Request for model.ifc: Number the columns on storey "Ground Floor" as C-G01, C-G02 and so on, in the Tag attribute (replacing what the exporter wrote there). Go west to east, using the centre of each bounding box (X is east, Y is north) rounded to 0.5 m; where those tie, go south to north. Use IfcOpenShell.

First a look at what the model holds.

```python
import ifcopenshell
import ifcopenshell.util.element
import ifcopenshell.util.placement

model = ifcopenshell.open("model.ifc")
print(model.schema)
storey = next(s for s in model.by_type("IfcBuildingStorey") if s.Name == "Ground Floor")
columns = [e for e in ifcopenshell.util.element.get_decomposition(storey) if e.is_a("IfcColumn")]
for e in sorted(columns, key=lambda e: e.id()):
    origin = ifcopenshell.util.placement.get_local_placement(e.ObjectPlacement)[:3, 3]
    print(e.id(), e.Tag, e.Name, origin.round(2) + 0.0, sep=" | ")
```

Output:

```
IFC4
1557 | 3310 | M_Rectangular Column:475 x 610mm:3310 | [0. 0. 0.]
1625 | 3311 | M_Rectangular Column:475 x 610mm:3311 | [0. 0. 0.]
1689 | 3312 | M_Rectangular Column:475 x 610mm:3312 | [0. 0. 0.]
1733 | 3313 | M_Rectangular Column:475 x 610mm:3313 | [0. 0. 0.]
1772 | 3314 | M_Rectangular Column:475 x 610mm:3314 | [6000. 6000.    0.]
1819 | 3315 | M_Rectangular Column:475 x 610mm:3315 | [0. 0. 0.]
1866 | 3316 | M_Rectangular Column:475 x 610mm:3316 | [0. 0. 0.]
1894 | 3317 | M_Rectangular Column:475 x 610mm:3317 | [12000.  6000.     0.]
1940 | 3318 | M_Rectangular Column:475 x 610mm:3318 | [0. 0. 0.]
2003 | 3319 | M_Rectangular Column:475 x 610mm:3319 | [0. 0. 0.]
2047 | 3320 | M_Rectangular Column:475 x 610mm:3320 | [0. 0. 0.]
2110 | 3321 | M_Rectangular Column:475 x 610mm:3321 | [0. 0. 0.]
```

```python
import ifcopenshell
import ifcopenshell.geom
import ifcopenshell.util.element
import ifcopenshell.util.shape

model = ifcopenshell.open("model.ifc")
settings = ifcopenshell.geom.settings()
settings.set("use-world-coords", True)


def centre(element):
    shape = ifcopenshell.geom.create_shape(settings, element)
    return ifcopenshell.util.shape.get_bbox_centroid(shape.geometry)


storey = next(s for s in model.by_type("IfcBuildingStorey") if s.Name == "Ground Floor")
columns = [e for e in ifcopenshell.util.element.get_decomposition(storey) if e.is_a("IfcColumn")]

# Insertion points can sit at a corner or the storey origin, so sort by the geometry (in metres).
centres = {e: centre(e) for e in columns}
columns.sort(key=lambda e: (round(centres[e][0] / 0.5), centres[e][1]))

for i, e in enumerate(columns, start=1):
    number = f"C-G{i:02d}"
    e.Tag = number
    print(e.id(), number)

model.write("model_edited.ifc")
```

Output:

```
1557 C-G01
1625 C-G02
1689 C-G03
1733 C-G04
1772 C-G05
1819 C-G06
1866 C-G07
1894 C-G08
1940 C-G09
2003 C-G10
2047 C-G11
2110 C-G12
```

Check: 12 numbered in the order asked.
